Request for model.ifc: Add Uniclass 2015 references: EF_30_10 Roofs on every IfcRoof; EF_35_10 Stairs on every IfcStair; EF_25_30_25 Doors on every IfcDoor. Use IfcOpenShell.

First a look at what the model holds.

```python
import ifcopenshell

model = ifcopenshell.open("model.ifc")
print(model.schema)
print("classifications:", [c.Name for c in model.by_type("IfcClassification")])
for ifc_class in ("IfcDoor", "IfcRoof", "IfcStair", "IfcWall", "IfcWindow"):
    print(ifc_class, len(model.by_type(ifc_class)))
```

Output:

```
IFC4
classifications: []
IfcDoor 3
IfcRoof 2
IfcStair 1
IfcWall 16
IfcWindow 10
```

```python
import ifcopenshell
import ifcopenshell.api.classification

model = ifcopenshell.open("model.ifc")

system = ifcopenshell.api.classification.add_classification(model, classification="Uniclass 2015")

codes = {
    "IfcRoof": ("EF_30_10", "Roofs"),
    "IfcStair": ("EF_35_10", "Stairs"),
    "IfcDoor": ("EF_25_30_25", "Doors"),
}
for ifc_class, (code, name) in codes.items():
    products = model.by_type(ifc_class)
    ifcopenshell.api.classification.add_reference(
        model, products=products, classification=system, identification=code, name=name
    )
    print(code, len(products))

model.write("model_updated.ifc")
```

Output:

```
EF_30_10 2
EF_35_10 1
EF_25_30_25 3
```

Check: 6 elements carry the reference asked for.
